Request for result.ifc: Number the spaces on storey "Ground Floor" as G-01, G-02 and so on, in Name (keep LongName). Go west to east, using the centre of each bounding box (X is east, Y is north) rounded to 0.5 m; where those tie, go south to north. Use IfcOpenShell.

First a look at what the model holds.

```python
import ifcopenshell
import ifcopenshell.util.element
import ifcopenshell.util.placement

model = ifcopenshell.open("result.ifc")
print(model.schema)
storey = next(s for s in model.by_type("IfcBuildingStorey") if s.Name == "Ground Floor")
spaces = [e for e in ifcopenshell.util.element.get_decomposition(storey) if e.is_a("IfcSpace")]
for e in sorted(spaces, key=lambda e: e.id()):
    origin = ifcopenshell.util.placement.get_local_placement(e.ObjectPlacement)[:3, 3]
    print(e.id(), e.Name, e.LongName, origin.round(2) + 0.0, sep=" | ")
```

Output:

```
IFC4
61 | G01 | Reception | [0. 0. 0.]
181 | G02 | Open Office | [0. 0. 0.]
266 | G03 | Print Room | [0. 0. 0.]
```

```python
import ifcopenshell
import ifcopenshell.geom
import ifcopenshell.util.element
import ifcopenshell.util.shape

model = ifcopenshell.open("result.ifc")
settings = ifcopenshell.geom.settings()
settings.set("use-world-coords", True)


def centre(element):
    shape = ifcopenshell.geom.create_shape(settings, element)
    return ifcopenshell.util.shape.get_bbox_centroid(shape.geometry)


storey = next(s for s in model.by_type("IfcBuildingStorey") if s.Name == "Ground Floor")
spaces = [e for e in ifcopenshell.util.element.get_decomposition(storey) if e.is_a("IfcSpace")]

# Insertion points can sit at a corner or the storey origin, so sort by the geometry (in metres).
centres = {e: centre(e) for e in spaces}
spaces.sort(key=lambda e: (round(centres[e][0] / 0.5), centres[e][1]))

for i, e in enumerate(spaces, start=1):
    number = f"G-{i:02d}"
    e.Name = number
    print(e.id(), number)

model.write("result_rev.ifc")
```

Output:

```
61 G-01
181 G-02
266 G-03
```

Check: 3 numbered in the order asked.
